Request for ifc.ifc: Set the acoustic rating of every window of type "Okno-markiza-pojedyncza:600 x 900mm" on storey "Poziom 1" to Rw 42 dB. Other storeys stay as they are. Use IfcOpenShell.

First a look at what the model holds.

```python
import ifcopenshell
import ifcopenshell.util.element

model = ifcopenshell.open("ifc.ifc")
print(model.schema)
storey = next(s for s in model.by_type("IfcBuildingStorey") if s.Name == "Poziom 1")
windows = [e for e in ifcopenshell.util.element.get_decomposition(storey) if e.is_a("IfcWindow")]
seen = {}
for e in windows:
    element_type = ifcopenshell.util.element.get_type(e)
    key = (element_type.Name if element_type != e and element_type else None, ifcopenshell.util.element.get_pset(e, "Pset_WindowCommon", "AcousticRating"))
    seen[key] = seen.get(key, 0) + 1
for (name, value), count in sorted(seen.items(), key=str):
    print(count, "x", name, "|", value)
```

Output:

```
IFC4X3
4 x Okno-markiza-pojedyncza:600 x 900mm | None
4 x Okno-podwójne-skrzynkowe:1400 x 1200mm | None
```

```python
import ifcopenshell
import ifcopenshell.api.pset
import ifcopenshell.util.element

model = ifcopenshell.open("ifc.ifc")

storey = next(s for s in model.by_type("IfcBuildingStorey") if s.Name == "Poziom 1")
windows = [e for e in ifcopenshell.util.element.get_decomposition(storey) if e.is_a("IfcWindow")]

count = 0
for e in windows:
    element_type = ifcopenshell.util.element.get_type(e)
    if element_type in (None, e) or element_type.Name != "Okno-markiza-pojedyncza:600 x 900mm":
        continue
    # add_pset returns the element's existing set when there is one.
    pset = ifcopenshell.api.pset.add_pset(model, product=e, name="Pset_WindowCommon")
    ifcopenshell.api.pset.edit_pset(model, pset=pset, properties={"AcousticRating": "Rw 42 dB"})
    count += 1

print(count, "windows updated")

model.write("ifc_rev.ifc")
```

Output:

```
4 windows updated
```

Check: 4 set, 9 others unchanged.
